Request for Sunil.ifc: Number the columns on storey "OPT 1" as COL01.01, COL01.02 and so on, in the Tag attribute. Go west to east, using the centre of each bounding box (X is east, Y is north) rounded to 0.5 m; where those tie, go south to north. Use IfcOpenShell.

First a look at what the model holds.

```python
import ifcopenshell
import ifcopenshell.util.element
import ifcopenshell.util.placement

model = ifcopenshell.open("Sunil.ifc")
print(model.schema)
storey = next(s for s in model.by_type("IfcBuildingStorey") if s.Name == "OPT 1")
columns = [e for e in ifcopenshell.util.element.get_decomposition(storey) if e.is_a("IfcColumn")]
for e in sorted(columns, key=lambda e: e.id()):
    origin = ifcopenshell.util.placement.get_local_placement(e.ObjectPlacement)[:3, 3]
    print(e.id(), e.Tag, e.Name, origin.round(2) + 0.0, sep=" | ")
```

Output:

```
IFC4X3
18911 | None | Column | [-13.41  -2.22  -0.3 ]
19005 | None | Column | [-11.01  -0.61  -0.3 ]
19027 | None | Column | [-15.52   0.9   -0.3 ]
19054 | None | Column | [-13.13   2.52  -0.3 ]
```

```python
import ifcopenshell
import ifcopenshell.geom
import ifcopenshell.util.element
import ifcopenshell.util.shape

model = ifcopenshell.open("Sunil.ifc")
settings = ifcopenshell.geom.settings()
settings.set("use-world-coords", True)


def centre(element):
    shape = ifcopenshell.geom.create_shape(settings, element)
    return ifcopenshell.util.shape.get_bbox_centroid(shape.geometry)


storey = next(s for s in model.by_type("IfcBuildingStorey") if s.Name == "OPT 1")
columns = [e for e in ifcopenshell.util.element.get_decomposition(storey) if e.is_a("IfcColumn")]

# Insertion points can sit at a corner or the storey origin, so sort by the geometry (in metres).
centres = {e: centre(e) for e in columns}
columns.sort(key=lambda e: (round(centres[e][0] / 0.5), centres[e][1]))

for i, e in enumerate(columns, start=1):
    number = f"COL01.{i:02d}"
    e.Tag = number
    print(e.id(), number)

model.write("Sunil_edited.ifc")
```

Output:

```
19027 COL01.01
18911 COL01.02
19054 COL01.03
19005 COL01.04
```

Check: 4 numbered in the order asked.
